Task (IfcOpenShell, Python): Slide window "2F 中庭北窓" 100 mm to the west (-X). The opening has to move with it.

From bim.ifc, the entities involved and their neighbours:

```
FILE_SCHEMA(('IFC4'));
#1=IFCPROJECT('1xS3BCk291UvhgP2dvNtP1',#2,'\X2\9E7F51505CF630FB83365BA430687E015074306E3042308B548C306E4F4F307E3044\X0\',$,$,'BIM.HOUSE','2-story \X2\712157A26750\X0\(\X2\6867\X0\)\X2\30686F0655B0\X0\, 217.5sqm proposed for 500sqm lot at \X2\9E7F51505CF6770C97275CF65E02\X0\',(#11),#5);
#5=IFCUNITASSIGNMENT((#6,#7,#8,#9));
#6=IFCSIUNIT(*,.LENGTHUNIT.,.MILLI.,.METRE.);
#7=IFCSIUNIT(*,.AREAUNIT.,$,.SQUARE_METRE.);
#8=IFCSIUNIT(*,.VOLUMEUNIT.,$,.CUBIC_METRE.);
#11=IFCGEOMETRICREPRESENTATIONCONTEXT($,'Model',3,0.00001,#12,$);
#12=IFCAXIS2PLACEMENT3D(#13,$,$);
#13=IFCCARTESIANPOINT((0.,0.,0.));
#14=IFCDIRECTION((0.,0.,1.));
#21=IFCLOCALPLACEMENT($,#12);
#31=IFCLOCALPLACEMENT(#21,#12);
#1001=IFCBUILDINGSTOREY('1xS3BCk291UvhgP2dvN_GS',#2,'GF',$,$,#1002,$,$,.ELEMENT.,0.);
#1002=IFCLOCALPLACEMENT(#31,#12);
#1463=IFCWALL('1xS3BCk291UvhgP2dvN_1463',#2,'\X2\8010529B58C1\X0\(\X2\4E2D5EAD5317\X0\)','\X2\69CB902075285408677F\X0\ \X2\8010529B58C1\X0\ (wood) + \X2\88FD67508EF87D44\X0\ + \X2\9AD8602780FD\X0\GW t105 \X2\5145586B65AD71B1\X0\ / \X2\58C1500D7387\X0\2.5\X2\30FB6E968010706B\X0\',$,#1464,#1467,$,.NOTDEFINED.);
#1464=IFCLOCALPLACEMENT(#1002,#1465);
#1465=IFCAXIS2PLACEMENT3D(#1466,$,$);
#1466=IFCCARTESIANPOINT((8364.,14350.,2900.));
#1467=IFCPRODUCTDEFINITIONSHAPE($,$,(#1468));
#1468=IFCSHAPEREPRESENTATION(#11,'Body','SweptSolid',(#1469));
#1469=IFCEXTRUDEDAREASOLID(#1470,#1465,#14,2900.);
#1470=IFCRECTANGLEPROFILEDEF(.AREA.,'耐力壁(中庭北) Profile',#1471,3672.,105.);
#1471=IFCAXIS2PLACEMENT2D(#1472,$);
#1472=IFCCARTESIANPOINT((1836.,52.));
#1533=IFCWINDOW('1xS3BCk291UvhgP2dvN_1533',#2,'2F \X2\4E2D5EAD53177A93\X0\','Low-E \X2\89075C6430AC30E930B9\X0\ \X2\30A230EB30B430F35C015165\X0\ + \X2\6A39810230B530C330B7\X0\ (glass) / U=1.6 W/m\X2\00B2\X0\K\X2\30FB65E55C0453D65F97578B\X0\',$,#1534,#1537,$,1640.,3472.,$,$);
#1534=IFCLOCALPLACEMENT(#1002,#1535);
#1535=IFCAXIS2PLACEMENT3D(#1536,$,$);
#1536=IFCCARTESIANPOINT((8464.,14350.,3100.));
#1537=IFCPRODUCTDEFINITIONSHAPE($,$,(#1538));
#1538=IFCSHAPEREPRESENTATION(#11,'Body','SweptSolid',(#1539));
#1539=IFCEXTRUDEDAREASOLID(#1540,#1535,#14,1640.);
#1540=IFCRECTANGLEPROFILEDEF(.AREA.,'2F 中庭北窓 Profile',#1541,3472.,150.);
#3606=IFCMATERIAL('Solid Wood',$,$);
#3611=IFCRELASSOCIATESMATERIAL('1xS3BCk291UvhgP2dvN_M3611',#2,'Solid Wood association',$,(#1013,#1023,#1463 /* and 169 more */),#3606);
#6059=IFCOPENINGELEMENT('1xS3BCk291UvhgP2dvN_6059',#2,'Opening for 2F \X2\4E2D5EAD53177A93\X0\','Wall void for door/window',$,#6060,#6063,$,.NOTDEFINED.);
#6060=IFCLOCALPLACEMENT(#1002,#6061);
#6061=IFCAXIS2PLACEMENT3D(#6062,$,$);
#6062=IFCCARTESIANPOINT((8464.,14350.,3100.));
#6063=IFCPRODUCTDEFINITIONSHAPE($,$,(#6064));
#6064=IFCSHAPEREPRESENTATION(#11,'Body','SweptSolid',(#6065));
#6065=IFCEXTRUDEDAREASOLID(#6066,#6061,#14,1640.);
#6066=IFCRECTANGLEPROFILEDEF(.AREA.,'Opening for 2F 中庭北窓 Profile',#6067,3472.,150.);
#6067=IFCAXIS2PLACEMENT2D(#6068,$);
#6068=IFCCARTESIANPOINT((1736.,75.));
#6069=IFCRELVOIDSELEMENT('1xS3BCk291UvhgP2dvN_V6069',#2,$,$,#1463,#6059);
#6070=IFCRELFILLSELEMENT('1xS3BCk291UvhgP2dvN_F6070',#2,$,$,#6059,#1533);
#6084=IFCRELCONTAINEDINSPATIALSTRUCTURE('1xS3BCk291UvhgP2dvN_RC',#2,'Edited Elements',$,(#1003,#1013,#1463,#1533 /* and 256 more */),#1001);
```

```python
import ifcopenshell
import ifcopenshell.api.geometry
import ifcopenshell.util.placement
import ifcopenshell.util.unit

model = ifcopenshell.open("bim.ifc")
unit_scale = ifcopenshell.util.unit.calculate_unit_scale(model)

window = model.by_guid("1xS3BCk291UvhgP2dvN_1533")
opening = window.FillsVoids[0].RelatingOpeningElement
wall = opening.VoidsElements[0].RelatingBuildingElement

wall_matrix = ifcopenshell.util.placement.get_local_placement(wall.ObjectPlacement)
shift = wall_matrix[:3, 0] * -0.1 / unit_scale
before = ifcopenshell.util.placement.get_local_placement(window.ObjectPlacement)[:3, 3].copy()

# The window is not placed relative to its opening, so move both.
for product in (opening, window):
    matrix = ifcopenshell.util.placement.get_local_placement(product.ObjectPlacement)
    matrix[:3, 3] += shift
    ifcopenshell.api.geometry.edit_object_placement(model, product=product, matrix=matrix, is_si=False)

after = ifcopenshell.util.placement.get_local_placement(window.ObjectPlacement)[:3, 3]
print("window moved by", (after - before).round(3) + 0.0)

model.write("bim_updated.ifc")
```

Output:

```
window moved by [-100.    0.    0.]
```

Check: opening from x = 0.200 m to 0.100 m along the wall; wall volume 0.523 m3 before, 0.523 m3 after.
